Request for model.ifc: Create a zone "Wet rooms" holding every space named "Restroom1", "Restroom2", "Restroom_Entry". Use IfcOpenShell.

First a look at what the model holds.

```python
import ifcopenshell

model = ifcopenshell.open("model.ifc")
print(model.schema)
seen = {}
for space in model.by_type("IfcSpace"):
    seen[space.LongName] = seen.get(space.LongName, 0) + 1
for name, count in sorted(seen.items(), key=str):
    print(count, "x", name)
print("zones:", [z.Name for z in model.by_type("IfcZone")][:20])
```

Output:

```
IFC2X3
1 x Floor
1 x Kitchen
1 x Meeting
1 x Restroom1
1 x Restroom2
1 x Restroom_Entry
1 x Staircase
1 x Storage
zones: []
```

```python
import ifcopenshell
import ifcopenshell.api.group
import ifcopenshell.api.root

model = ifcopenshell.open("model.ifc")

names = {"Restroom1", "Restroom2", "Restroom_Entry"}
spaces = [s for s in model.by_type("IfcSpace") if s.LongName in names]

zone = ifcopenshell.api.root.create_entity(model, ifc_class="IfcZone", name="Wet rooms")
ifcopenshell.api.group.assign_group(model, products=spaces, group=zone)
print(len(spaces), "spaces in", zone.Name)

model.write("model-out.ifc")
```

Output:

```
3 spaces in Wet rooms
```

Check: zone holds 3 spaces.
